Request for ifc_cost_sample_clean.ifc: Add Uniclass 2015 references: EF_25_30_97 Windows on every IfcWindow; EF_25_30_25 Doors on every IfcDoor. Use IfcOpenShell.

First a look at what the model holds.

```python
import ifcopenshell

model = ifcopenshell.open("ifc_cost_sample_clean.ifc")
print(model.schema)
print("classifications:", [c.Name for c in model.by_type("IfcClassification")])
for ifc_class in ("IfcDoor", "IfcRoof", "IfcStair", "IfcWall", "IfcWindow"):
    print(ifc_class, len(model.by_type(ifc_class)))
```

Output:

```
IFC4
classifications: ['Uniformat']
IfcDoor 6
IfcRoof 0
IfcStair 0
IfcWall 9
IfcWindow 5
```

```python
import ifcopenshell
import ifcopenshell.api.classification

model = ifcopenshell.open("ifc_cost_sample_clean.ifc")

system = ifcopenshell.api.classification.add_classification(model, classification="Uniclass 2015")

codes = {
    "IfcWindow": ("EF_25_30_97", "Windows"),
    "IfcDoor": ("EF_25_30_25", "Doors"),
}
for ifc_class, (code, name) in codes.items():
    products = model.by_type(ifc_class)
    ifcopenshell.api.classification.add_reference(
        model, products=products, classification=system, identification=code, name=name
    )
    print(code, len(products))

model.write("ifc_cost_sample_clean-out.ifc")
```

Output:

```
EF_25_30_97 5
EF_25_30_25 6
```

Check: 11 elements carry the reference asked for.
